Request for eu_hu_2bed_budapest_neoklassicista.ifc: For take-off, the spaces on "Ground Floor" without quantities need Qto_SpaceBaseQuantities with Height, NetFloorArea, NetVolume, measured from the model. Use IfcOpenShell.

First a look at what the model holds.

```python
import ifcopenshell
import ifcopenshell.util.element
import ifcopenshell.util.unit

model = ifcopenshell.open("eu_hu_2bed_budapest_neoklassicista.ifc")
print(model.schema)
for unit_type in ("LENGTHUNIT", "AREAUNIT", "VOLUMEUNIT"):
    print(unit_type, ifcopenshell.util.unit.calculate_unit_scale(model, unit_type))
storey = next(s for s in model.by_type("IfcBuildingStorey") if s.Name == "Ground Floor")
spaces = [e for e in ifcopenshell.util.element.get_decomposition(storey) if e.is_a("IfcSpace")]
for e in sorted(spaces, key=lambda e: e.id()):
    print(e.id(), e.is_a(), e.Name, list(ifcopenshell.util.element.get_psets(e, qtos_only=True)), sep=" | ")
```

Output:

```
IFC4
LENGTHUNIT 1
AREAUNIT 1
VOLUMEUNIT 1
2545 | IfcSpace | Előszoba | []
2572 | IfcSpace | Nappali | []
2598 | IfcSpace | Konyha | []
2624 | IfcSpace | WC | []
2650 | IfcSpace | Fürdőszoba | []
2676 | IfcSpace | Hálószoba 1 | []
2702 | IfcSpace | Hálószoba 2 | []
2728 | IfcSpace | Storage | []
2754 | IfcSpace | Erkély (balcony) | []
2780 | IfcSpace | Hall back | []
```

```python
import ifcopenshell
import ifcopenshell.api.pset
import ifcopenshell.geom
import ifcopenshell.util.element
import ifcopenshell.util.shape
import ifcopenshell.util.unit

model = ifcopenshell.open("eu_hu_2bed_budapest_neoklassicista.ifc")
unit_scale = ifcopenshell.util.unit.calculate_unit_scale(model)
area_scale = ifcopenshell.util.unit.calculate_unit_scale(model, "AREAUNIT")
volume_scale = ifcopenshell.util.unit.calculate_unit_scale(model, "VOLUMEUNIT")
settings = ifcopenshell.geom.settings()

storey = next(s for s in model.by_type("IfcBuildingStorey") if s.Name == "Ground Floor")
spaces = [e for e in ifcopenshell.util.element.get_decomposition(storey) if e.is_a("IfcSpace")]

for e in sorted(spaces, key=lambda e: e.id()):
    if ifcopenshell.util.element.get_psets(e, qtos_only=True, should_inherit=False):
        continue
    # Geometry comes back in metres, in the element's own axes.
    shape = ifcopenshell.geom.create_shape(settings, e)
    values = {
        "Height": ifcopenshell.util.shape.get_z(shape.geometry) / unit_scale,
        "NetFloorArea": ifcopenshell.util.shape.get_footprint_area(shape.geometry) / area_scale,
        "NetVolume": ifcopenshell.util.shape.get_volume(shape.geometry) / volume_scale,
    }
    qto = ifcopenshell.api.pset.add_qto(model, product=e, name="Qto_SpaceBaseQuantities")
    ifcopenshell.api.pset.edit_qto(model, qto=qto, properties=values)
    print(e.id(), {k: round(v, 3) for k, v in values.items()})

model.write("eu_hu_2bed_budapest_neoklassicista_edited.ifc")
```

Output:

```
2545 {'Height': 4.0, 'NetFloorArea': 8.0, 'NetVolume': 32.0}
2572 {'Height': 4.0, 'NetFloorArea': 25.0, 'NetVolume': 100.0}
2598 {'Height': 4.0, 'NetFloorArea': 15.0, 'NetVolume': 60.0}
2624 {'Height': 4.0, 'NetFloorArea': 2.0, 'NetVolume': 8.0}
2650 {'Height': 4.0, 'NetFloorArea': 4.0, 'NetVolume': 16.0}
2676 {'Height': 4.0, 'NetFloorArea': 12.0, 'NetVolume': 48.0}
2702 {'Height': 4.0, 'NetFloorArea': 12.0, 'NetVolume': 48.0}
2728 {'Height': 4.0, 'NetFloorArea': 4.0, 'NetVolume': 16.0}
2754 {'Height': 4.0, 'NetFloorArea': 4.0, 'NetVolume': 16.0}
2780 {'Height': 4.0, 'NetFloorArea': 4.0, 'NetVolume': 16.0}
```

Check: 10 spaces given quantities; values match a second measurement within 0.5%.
